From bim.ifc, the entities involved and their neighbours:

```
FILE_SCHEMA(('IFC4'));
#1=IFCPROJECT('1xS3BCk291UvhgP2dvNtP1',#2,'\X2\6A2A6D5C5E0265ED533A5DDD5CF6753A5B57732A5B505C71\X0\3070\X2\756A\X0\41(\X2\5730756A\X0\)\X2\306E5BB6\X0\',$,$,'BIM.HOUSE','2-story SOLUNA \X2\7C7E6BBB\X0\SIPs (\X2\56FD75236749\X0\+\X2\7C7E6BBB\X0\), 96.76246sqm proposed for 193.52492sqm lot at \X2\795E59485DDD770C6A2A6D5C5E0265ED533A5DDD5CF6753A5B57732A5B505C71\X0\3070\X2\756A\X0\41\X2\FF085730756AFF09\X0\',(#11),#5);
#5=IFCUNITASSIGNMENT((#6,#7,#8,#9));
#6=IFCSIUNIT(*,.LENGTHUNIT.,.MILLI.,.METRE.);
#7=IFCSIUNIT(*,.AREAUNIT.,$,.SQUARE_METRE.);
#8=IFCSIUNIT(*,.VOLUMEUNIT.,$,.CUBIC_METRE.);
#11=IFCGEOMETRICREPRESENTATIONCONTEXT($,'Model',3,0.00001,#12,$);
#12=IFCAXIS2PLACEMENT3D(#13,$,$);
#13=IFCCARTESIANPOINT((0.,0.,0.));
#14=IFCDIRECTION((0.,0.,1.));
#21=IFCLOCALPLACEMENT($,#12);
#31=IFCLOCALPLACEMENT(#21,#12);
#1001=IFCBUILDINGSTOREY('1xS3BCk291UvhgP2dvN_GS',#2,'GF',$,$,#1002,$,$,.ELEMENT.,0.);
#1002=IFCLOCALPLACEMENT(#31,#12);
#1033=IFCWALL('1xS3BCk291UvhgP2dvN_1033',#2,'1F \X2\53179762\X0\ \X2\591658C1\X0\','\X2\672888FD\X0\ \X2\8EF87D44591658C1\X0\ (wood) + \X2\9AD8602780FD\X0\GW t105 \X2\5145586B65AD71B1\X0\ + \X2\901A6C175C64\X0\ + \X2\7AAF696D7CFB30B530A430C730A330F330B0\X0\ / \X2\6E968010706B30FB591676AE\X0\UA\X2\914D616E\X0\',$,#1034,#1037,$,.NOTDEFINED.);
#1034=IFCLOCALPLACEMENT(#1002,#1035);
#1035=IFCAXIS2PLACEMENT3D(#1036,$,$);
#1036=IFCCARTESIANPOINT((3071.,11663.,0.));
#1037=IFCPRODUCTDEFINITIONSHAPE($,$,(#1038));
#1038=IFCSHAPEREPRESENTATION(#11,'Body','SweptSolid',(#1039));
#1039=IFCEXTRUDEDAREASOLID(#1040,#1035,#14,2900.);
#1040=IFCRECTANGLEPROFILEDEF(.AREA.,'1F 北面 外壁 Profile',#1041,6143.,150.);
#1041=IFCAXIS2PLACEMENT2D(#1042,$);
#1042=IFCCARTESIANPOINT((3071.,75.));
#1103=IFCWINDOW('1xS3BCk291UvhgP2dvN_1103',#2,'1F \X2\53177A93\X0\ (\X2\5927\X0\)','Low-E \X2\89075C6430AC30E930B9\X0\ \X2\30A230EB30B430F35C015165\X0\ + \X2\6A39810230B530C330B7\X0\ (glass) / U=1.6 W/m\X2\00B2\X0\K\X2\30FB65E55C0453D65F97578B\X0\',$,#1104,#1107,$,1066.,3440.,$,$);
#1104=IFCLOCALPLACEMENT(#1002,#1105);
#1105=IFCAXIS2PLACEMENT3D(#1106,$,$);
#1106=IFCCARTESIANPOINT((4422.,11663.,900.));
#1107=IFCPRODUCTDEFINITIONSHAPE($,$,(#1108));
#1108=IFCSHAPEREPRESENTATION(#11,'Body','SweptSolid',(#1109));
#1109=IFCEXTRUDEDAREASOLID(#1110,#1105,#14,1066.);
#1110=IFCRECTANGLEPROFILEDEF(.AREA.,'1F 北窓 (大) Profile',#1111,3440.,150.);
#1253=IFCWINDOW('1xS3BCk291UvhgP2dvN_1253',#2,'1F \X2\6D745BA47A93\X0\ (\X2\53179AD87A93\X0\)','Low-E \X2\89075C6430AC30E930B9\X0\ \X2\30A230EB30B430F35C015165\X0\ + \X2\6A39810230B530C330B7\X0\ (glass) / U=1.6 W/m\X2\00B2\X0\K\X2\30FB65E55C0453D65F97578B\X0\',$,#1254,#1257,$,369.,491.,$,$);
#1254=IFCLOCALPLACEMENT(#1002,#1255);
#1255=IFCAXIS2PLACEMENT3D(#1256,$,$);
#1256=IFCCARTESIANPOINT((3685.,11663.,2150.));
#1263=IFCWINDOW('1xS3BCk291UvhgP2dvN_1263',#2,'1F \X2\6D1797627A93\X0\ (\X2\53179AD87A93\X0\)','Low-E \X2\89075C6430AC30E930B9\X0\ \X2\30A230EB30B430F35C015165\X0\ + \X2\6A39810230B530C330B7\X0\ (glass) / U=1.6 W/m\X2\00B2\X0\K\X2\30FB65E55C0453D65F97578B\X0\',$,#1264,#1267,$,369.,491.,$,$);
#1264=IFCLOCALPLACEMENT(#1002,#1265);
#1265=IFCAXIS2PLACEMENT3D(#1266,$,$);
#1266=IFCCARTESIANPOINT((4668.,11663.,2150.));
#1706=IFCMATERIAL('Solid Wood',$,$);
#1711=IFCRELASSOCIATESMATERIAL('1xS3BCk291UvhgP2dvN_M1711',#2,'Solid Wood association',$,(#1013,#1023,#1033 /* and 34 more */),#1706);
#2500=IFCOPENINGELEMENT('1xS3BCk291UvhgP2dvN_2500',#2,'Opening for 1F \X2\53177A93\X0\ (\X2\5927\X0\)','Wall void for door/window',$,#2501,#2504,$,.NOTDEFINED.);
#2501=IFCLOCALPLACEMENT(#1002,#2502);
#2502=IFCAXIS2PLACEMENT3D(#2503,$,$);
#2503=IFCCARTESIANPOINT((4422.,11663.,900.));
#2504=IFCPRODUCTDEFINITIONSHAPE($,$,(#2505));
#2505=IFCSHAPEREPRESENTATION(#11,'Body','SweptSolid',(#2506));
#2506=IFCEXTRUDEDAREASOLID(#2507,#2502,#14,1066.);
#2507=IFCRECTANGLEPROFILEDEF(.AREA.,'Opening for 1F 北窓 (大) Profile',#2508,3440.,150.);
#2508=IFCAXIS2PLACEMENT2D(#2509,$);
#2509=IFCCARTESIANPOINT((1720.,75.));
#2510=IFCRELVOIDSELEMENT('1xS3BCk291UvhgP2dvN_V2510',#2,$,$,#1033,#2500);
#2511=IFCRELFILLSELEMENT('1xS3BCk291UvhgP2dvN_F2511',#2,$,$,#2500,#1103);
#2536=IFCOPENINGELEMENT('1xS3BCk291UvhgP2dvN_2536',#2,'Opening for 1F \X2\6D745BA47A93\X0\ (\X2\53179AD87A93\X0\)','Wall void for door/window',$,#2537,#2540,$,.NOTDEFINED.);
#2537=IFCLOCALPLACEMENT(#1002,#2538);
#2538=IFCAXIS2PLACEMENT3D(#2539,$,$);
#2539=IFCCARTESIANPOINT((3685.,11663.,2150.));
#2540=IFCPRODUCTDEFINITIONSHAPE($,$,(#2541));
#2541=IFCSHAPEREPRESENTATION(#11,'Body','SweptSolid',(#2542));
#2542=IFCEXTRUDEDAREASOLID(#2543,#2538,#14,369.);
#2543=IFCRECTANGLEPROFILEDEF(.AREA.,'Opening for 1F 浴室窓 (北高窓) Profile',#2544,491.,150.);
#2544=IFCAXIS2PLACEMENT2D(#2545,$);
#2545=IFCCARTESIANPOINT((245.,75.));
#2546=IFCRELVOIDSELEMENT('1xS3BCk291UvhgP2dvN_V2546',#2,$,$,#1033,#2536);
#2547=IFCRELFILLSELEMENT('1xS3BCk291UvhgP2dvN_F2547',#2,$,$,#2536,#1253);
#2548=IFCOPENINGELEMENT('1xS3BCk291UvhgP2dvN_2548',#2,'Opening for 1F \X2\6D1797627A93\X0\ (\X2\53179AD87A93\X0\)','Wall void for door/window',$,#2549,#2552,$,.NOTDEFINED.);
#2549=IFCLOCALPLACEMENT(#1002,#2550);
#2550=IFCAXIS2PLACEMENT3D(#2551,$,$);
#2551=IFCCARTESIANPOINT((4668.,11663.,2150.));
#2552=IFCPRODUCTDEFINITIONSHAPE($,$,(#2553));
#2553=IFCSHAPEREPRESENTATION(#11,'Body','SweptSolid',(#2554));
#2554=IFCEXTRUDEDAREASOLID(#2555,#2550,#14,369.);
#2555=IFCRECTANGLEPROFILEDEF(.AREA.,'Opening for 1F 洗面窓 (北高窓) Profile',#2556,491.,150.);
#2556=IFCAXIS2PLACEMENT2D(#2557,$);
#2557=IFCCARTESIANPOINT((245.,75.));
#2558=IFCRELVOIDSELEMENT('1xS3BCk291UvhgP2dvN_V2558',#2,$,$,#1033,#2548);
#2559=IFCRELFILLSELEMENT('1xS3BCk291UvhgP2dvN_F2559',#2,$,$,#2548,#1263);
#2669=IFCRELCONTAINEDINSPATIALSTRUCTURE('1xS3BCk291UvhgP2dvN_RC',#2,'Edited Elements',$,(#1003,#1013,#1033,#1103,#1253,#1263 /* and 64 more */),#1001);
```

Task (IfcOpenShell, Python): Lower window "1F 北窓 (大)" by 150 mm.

```python
import numpy as np
import ifcopenshell
import ifcopenshell.api.geometry
import ifcopenshell.util.placement
import ifcopenshell.util.unit

model = ifcopenshell.open("bim.ifc")
unit_scale = ifcopenshell.util.unit.calculate_unit_scale(model)

window = model.by_guid("1xS3BCk291UvhgP2dvN_1103")
opening = window.FillsVoids[0].RelatingOpeningElement
dz = -150.0

shift = np.array([0.0, 0.0, dz])
# The window is not placed relative to its opening, so move both.
for product in (opening, window):
    matrix = ifcopenshell.util.placement.get_local_placement(product.ObjectPlacement)
    matrix[:3, 3] += shift
    ifcopenshell.api.geometry.edit_object_placement(model, product=product, matrix=matrix, is_si=False)

print(f"moved by {dz * unit_scale:+.3f} m")

model.write("bim_edited.ifc")
```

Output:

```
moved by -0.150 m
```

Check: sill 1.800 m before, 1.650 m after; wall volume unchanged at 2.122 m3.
